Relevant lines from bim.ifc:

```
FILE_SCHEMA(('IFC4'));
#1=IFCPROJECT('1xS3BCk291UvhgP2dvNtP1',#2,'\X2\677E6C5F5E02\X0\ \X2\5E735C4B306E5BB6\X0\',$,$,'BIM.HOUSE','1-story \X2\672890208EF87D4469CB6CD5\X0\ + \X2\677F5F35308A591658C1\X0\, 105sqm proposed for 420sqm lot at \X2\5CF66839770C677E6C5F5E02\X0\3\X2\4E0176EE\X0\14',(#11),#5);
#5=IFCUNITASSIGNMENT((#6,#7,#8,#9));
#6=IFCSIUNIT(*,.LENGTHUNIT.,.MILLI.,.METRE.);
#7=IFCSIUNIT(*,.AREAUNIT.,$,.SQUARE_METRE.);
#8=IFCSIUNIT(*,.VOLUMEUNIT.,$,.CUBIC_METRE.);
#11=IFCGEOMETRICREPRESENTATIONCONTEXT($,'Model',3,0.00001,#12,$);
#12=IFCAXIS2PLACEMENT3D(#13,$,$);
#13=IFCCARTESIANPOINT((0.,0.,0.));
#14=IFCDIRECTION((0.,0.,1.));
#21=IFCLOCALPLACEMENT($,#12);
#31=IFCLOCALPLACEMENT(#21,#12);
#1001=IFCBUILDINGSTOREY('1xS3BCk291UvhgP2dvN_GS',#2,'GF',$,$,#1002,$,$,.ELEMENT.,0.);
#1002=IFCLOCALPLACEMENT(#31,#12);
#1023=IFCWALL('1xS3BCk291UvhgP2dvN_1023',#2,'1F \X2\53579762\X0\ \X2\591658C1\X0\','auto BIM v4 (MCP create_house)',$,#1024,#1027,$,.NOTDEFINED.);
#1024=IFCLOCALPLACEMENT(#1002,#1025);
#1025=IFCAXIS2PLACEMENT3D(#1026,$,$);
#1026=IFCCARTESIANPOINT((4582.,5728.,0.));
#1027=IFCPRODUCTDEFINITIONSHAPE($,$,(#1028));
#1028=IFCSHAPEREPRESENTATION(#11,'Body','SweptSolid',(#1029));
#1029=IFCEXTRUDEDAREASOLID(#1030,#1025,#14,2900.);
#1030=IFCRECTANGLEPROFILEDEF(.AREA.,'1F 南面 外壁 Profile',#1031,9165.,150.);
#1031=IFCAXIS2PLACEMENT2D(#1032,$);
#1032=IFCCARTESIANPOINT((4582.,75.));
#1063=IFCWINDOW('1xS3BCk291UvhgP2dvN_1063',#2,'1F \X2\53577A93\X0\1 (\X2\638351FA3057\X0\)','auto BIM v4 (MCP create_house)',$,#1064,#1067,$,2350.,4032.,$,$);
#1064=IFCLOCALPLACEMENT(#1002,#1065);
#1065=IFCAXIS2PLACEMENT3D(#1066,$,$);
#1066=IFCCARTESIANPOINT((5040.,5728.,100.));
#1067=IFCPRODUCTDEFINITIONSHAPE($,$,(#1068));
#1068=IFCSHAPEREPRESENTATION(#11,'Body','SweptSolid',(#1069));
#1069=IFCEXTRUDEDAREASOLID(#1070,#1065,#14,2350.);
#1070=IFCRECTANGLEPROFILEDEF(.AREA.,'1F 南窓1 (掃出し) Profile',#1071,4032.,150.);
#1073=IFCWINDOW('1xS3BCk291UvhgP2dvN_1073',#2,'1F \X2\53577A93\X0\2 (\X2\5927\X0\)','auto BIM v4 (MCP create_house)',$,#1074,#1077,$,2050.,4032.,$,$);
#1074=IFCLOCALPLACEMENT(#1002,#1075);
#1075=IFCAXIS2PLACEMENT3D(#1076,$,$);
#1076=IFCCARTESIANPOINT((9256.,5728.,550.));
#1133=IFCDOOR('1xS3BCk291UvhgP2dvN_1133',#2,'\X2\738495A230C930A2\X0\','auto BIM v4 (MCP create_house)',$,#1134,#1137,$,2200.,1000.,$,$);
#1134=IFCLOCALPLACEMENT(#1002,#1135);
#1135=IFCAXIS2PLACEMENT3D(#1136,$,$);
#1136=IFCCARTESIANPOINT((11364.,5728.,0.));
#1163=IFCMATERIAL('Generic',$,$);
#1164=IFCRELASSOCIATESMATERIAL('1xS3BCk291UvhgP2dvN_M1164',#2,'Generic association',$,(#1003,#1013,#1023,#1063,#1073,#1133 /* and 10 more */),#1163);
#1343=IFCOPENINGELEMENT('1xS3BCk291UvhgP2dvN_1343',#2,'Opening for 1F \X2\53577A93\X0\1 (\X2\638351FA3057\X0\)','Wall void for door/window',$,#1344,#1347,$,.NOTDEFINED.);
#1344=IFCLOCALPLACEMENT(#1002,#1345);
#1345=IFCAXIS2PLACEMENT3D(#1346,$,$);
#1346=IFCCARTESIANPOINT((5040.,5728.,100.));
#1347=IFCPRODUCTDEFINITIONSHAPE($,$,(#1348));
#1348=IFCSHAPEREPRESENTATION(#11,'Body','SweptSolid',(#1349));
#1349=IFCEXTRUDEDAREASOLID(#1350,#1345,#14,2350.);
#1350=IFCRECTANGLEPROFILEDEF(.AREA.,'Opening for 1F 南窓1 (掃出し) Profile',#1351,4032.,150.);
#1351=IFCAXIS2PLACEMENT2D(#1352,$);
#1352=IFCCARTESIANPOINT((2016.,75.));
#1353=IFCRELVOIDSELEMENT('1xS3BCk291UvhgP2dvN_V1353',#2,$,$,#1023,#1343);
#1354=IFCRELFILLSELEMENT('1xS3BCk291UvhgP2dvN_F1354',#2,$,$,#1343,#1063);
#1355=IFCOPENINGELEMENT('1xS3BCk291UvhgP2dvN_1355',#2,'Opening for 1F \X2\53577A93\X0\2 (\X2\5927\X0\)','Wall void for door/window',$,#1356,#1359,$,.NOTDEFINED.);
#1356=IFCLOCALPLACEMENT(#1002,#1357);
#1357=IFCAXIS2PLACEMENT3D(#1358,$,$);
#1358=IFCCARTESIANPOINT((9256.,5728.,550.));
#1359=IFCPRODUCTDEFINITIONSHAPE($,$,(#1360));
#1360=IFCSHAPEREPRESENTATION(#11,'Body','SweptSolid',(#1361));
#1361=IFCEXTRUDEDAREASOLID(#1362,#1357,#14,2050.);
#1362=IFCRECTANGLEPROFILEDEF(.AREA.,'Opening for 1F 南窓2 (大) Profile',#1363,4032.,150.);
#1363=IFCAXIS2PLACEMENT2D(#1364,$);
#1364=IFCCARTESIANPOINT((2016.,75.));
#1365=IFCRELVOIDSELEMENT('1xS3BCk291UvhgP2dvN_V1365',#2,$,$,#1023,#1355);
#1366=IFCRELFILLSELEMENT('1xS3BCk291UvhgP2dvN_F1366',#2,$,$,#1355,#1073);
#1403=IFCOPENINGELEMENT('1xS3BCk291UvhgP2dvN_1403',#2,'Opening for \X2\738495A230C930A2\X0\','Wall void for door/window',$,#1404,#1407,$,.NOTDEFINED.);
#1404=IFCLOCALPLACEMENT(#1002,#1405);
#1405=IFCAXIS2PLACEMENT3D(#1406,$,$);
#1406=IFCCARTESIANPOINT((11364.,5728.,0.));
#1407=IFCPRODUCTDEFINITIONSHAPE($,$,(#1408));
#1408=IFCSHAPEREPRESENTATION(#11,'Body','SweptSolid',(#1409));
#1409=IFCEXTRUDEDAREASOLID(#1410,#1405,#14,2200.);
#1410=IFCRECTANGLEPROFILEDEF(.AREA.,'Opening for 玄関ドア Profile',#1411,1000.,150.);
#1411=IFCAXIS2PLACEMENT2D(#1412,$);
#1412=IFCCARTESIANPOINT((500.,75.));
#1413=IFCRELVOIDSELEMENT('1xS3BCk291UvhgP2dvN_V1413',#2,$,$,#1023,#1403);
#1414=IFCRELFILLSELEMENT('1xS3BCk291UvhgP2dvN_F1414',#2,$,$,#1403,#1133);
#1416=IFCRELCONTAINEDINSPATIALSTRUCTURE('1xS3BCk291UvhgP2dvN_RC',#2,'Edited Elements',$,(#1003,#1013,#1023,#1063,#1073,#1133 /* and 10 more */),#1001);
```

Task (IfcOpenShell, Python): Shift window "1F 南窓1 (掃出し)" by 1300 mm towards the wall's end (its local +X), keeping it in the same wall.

```python
import ifcopenshell
import ifcopenshell.api.geometry
import ifcopenshell.util.placement
import ifcopenshell.util.unit

model = ifcopenshell.open("bim.ifc")
unit_scale = ifcopenshell.util.unit.calculate_unit_scale(model)

window = model.by_id(1063)
opening = window.FillsVoids[0].RelatingOpeningElement
wall = opening.VoidsElements[0].RelatingBuildingElement

wall_matrix = ifcopenshell.util.placement.get_local_placement(wall.ObjectPlacement)
shift = wall_matrix[:3, 0] * 1.3 / unit_scale
before = ifcopenshell.util.placement.get_local_placement(window.ObjectPlacement)[:3, 3].copy()

# The window is not placed relative to its opening, so move both.
for product in (opening, window):
    matrix = ifcopenshell.util.placement.get_local_placement(product.ObjectPlacement)
    matrix[:3, 3] += shift
    ifcopenshell.api.geometry.edit_object_placement(model, product=product, matrix=matrix, is_si=False)

after = ifcopenshell.util.placement.get_local_placement(window.ObjectPlacement)[:3, 3]
print("window moved by", (after - before).round(3) + 0.0)

model.write("bim_rev.ifc")
```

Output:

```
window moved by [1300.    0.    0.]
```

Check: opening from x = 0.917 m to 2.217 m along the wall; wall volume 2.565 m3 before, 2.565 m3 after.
